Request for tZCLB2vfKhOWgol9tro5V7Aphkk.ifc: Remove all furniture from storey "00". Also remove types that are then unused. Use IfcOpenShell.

First a look at what the model holds.

```python
import ifcopenshell
import ifcopenshell.util.element

model = ifcopenshell.open("tZCLB2vfKhOWgol9tro5V7Aphkk.ifc")
print(model.schema)
storey = next(s for s in model.by_type("IfcBuildingStorey") if s.Name == "00")
furniture = [e for e in ifcopenshell.util.element.get_decomposition(storey) if e.is_a("IfcFurnishingElement")]
seen = {}
for e in furniture:
    element_type = ifcopenshell.util.element.get_type(e)
    name = element_type.Name if element_type not in (None, e) else None
    seen[name] = seen.get(name, 0) + 1
for name, count in sorted(seen.items(), key=str):
    print(count, "x", name)
```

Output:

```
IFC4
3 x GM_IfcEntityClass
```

```python
import ifcopenshell
import ifcopenshell.api.root
import ifcopenshell.util.element

model = ifcopenshell.open("tZCLB2vfKhOWgol9tro5V7Aphkk.ifc")

storey = next(s for s in model.by_type("IfcBuildingStorey") if s.Name == "00")
furniture = [e for e in ifcopenshell.util.element.get_decomposition(storey) if e.is_a("IfcFurnishingElement")]
types = {ifcopenshell.util.element.get_type(e) for e in furniture} - {None, *furniture}

for e in furniture:
    ifcopenshell.api.root.remove_product(model, product=e)
print(len(furniture), "removed")

unused = [t for t in types if not ifcopenshell.util.element.get_types(t)]
for t in unused:
    ifcopenshell.api.root.remove_product(model, product=t)
print(len(unused), "unused types removed")

model.write("tZCLB2vfKhOWgol9tro5V7Aphkk_updated.ifc")
```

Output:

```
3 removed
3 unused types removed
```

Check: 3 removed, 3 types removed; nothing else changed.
